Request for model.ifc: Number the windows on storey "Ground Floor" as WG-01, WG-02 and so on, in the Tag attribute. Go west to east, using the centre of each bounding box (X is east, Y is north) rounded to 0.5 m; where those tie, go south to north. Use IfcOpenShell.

First a look at what the model holds.

```python
import ifcopenshell
import ifcopenshell.util.element
import ifcopenshell.util.placement

model = ifcopenshell.open("model.ifc")
print(model.schema)
storey = next(s for s in model.by_type("IfcBuildingStorey") if s.Name == "Ground Floor")
windows = [e for e in ifcopenshell.util.element.get_decomposition(storey) if e.is_a("IfcWindow")]
for e in sorted(windows, key=lambda e: e.id()):
    origin = ifcopenshell.util.placement.get_local_placement(e.ObjectPlacement)[:3, 3]
    print(e.id(), e.Tag, e.Name, origin.round(2) + 0.0, sep=" | ")
```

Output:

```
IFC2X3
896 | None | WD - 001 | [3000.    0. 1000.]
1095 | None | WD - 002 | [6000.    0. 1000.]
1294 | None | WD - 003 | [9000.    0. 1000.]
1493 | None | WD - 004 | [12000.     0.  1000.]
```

```python
import ifcopenshell
import ifcopenshell.geom
import ifcopenshell.util.element
import ifcopenshell.util.shape

model = ifcopenshell.open("model.ifc")
settings = ifcopenshell.geom.settings()
settings.set("use-world-coords", True)


def centre(element):
    shape = ifcopenshell.geom.create_shape(settings, element)
    return ifcopenshell.util.shape.get_bbox_centroid(shape.geometry)


storey = next(s for s in model.by_type("IfcBuildingStorey") if s.Name == "Ground Floor")
windows = [e for e in ifcopenshell.util.element.get_decomposition(storey) if e.is_a("IfcWindow")]

# Insertion points can sit at a corner or the storey origin, so sort by the geometry (in metres).
centres = {e: centre(e) for e in windows}
windows.sort(key=lambda e: (round(centres[e][0] / 0.5), centres[e][1]))

for i, e in enumerate(windows, start=1):
    number = f"WG-{i:02d}"
    e.Tag = number
    print(e.id(), number)

model.write("model_v2.ifc")
```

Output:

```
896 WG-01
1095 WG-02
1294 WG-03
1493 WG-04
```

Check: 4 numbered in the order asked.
